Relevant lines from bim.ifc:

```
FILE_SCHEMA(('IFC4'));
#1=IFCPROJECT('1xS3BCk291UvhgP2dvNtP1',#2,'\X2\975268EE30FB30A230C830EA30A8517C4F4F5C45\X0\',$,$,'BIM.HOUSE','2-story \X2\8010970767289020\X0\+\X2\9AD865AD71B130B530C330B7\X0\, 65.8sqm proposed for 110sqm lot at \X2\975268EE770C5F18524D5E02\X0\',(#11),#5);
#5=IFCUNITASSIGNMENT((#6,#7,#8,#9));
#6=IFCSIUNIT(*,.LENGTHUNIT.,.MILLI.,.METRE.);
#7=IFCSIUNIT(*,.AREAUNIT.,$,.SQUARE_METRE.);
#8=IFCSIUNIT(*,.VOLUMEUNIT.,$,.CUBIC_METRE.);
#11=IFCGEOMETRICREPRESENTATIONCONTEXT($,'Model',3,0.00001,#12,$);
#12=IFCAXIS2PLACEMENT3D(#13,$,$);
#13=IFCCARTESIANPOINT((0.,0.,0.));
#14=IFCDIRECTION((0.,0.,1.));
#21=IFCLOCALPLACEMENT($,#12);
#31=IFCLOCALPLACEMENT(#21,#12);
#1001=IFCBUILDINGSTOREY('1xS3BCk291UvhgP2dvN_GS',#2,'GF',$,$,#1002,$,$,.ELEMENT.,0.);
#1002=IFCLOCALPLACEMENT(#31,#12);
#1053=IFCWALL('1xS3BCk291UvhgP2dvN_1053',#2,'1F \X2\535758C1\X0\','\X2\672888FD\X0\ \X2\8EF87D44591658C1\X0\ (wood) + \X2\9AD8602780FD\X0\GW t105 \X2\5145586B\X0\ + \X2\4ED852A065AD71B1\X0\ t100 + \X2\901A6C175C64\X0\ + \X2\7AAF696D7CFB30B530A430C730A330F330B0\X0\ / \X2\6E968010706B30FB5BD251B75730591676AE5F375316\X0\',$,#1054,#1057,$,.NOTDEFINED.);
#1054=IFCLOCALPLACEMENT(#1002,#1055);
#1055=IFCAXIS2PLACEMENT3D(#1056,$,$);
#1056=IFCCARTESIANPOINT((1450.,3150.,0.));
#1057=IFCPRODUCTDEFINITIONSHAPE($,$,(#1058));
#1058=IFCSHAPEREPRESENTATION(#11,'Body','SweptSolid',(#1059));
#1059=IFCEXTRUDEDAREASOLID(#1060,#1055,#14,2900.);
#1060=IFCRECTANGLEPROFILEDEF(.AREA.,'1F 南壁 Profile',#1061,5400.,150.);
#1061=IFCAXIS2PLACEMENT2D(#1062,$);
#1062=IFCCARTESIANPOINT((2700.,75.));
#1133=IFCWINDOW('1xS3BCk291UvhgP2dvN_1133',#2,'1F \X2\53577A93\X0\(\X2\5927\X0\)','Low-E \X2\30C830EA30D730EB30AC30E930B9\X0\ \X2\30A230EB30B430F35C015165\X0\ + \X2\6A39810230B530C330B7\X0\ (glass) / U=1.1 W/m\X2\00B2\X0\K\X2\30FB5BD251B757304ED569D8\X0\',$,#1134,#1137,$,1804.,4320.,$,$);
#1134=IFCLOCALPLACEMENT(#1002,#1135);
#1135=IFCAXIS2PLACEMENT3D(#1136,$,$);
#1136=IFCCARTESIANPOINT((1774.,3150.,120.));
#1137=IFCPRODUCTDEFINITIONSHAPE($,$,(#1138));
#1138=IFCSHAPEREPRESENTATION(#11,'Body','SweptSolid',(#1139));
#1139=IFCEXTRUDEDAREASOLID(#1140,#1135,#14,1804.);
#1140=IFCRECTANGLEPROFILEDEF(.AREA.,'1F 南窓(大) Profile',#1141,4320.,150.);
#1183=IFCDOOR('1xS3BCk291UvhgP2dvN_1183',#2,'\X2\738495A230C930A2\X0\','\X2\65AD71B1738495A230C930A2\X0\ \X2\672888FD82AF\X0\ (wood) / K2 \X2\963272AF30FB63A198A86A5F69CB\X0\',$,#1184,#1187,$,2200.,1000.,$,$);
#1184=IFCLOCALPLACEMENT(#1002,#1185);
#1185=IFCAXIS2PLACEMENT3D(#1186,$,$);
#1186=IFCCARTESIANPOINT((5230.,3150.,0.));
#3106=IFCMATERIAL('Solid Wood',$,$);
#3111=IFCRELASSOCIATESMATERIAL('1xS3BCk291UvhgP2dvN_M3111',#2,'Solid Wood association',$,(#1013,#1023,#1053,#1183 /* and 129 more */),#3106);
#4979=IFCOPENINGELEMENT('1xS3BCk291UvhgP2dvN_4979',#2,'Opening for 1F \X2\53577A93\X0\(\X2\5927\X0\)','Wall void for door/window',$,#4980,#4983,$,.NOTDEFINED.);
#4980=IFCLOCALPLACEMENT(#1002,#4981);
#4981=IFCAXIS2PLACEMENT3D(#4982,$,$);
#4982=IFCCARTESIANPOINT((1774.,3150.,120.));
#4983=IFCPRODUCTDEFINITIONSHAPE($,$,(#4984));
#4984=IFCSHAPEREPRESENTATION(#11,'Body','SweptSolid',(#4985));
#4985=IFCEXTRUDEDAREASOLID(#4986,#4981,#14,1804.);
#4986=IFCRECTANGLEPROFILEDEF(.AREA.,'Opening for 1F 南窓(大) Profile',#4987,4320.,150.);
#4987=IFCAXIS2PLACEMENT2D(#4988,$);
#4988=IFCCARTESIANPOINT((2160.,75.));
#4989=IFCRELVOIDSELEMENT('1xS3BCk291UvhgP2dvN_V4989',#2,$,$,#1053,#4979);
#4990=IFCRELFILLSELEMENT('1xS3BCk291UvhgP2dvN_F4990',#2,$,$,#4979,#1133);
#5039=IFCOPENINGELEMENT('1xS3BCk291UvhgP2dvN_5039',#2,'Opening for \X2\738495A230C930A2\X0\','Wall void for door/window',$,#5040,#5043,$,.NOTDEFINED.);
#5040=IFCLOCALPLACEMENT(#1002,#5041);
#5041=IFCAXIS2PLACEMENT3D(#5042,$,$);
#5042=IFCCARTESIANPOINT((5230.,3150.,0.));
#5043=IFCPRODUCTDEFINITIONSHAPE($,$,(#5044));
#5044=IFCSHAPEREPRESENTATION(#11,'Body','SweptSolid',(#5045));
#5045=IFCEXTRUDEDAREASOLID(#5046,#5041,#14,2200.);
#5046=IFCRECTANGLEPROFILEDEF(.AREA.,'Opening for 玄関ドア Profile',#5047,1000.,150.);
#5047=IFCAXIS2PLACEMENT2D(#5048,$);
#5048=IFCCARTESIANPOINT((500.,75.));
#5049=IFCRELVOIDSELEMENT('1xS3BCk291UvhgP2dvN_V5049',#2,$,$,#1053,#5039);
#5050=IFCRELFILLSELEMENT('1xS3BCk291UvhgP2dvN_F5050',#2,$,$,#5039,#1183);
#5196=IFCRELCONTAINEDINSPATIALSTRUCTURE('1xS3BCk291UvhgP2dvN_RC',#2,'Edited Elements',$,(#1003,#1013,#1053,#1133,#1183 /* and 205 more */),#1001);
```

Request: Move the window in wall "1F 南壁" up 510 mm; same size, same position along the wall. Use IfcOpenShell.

```python
import numpy as np
import ifcopenshell
import ifcopenshell.api.geometry
import ifcopenshell.util.placement
import ifcopenshell.util.unit

model = ifcopenshell.open("bim.ifc")
unit_scale = ifcopenshell.util.unit.calculate_unit_scale(model)

window = model.by_guid("1xS3BCk291UvhgP2dvN_1133")
opening = window.FillsVoids[0].RelatingOpeningElement
dz = 0.51 / unit_scale

shift = np.array([0.0, 0.0, dz])
# The window is not placed relative to its opening, so move both.
for product in (opening, window):
    matrix = ifcopenshell.util.placement.get_local_placement(product.ObjectPlacement)
    matrix[:3, 3] += shift
    ifcopenshell.api.geometry.edit_object_placement(model, product=product, matrix=matrix, is_si=False)

print(f"moved by {dz * unit_scale:+.3f} m")

model.write("bim_v2.ifc")
```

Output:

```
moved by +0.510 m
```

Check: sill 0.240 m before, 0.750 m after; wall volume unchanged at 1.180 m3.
